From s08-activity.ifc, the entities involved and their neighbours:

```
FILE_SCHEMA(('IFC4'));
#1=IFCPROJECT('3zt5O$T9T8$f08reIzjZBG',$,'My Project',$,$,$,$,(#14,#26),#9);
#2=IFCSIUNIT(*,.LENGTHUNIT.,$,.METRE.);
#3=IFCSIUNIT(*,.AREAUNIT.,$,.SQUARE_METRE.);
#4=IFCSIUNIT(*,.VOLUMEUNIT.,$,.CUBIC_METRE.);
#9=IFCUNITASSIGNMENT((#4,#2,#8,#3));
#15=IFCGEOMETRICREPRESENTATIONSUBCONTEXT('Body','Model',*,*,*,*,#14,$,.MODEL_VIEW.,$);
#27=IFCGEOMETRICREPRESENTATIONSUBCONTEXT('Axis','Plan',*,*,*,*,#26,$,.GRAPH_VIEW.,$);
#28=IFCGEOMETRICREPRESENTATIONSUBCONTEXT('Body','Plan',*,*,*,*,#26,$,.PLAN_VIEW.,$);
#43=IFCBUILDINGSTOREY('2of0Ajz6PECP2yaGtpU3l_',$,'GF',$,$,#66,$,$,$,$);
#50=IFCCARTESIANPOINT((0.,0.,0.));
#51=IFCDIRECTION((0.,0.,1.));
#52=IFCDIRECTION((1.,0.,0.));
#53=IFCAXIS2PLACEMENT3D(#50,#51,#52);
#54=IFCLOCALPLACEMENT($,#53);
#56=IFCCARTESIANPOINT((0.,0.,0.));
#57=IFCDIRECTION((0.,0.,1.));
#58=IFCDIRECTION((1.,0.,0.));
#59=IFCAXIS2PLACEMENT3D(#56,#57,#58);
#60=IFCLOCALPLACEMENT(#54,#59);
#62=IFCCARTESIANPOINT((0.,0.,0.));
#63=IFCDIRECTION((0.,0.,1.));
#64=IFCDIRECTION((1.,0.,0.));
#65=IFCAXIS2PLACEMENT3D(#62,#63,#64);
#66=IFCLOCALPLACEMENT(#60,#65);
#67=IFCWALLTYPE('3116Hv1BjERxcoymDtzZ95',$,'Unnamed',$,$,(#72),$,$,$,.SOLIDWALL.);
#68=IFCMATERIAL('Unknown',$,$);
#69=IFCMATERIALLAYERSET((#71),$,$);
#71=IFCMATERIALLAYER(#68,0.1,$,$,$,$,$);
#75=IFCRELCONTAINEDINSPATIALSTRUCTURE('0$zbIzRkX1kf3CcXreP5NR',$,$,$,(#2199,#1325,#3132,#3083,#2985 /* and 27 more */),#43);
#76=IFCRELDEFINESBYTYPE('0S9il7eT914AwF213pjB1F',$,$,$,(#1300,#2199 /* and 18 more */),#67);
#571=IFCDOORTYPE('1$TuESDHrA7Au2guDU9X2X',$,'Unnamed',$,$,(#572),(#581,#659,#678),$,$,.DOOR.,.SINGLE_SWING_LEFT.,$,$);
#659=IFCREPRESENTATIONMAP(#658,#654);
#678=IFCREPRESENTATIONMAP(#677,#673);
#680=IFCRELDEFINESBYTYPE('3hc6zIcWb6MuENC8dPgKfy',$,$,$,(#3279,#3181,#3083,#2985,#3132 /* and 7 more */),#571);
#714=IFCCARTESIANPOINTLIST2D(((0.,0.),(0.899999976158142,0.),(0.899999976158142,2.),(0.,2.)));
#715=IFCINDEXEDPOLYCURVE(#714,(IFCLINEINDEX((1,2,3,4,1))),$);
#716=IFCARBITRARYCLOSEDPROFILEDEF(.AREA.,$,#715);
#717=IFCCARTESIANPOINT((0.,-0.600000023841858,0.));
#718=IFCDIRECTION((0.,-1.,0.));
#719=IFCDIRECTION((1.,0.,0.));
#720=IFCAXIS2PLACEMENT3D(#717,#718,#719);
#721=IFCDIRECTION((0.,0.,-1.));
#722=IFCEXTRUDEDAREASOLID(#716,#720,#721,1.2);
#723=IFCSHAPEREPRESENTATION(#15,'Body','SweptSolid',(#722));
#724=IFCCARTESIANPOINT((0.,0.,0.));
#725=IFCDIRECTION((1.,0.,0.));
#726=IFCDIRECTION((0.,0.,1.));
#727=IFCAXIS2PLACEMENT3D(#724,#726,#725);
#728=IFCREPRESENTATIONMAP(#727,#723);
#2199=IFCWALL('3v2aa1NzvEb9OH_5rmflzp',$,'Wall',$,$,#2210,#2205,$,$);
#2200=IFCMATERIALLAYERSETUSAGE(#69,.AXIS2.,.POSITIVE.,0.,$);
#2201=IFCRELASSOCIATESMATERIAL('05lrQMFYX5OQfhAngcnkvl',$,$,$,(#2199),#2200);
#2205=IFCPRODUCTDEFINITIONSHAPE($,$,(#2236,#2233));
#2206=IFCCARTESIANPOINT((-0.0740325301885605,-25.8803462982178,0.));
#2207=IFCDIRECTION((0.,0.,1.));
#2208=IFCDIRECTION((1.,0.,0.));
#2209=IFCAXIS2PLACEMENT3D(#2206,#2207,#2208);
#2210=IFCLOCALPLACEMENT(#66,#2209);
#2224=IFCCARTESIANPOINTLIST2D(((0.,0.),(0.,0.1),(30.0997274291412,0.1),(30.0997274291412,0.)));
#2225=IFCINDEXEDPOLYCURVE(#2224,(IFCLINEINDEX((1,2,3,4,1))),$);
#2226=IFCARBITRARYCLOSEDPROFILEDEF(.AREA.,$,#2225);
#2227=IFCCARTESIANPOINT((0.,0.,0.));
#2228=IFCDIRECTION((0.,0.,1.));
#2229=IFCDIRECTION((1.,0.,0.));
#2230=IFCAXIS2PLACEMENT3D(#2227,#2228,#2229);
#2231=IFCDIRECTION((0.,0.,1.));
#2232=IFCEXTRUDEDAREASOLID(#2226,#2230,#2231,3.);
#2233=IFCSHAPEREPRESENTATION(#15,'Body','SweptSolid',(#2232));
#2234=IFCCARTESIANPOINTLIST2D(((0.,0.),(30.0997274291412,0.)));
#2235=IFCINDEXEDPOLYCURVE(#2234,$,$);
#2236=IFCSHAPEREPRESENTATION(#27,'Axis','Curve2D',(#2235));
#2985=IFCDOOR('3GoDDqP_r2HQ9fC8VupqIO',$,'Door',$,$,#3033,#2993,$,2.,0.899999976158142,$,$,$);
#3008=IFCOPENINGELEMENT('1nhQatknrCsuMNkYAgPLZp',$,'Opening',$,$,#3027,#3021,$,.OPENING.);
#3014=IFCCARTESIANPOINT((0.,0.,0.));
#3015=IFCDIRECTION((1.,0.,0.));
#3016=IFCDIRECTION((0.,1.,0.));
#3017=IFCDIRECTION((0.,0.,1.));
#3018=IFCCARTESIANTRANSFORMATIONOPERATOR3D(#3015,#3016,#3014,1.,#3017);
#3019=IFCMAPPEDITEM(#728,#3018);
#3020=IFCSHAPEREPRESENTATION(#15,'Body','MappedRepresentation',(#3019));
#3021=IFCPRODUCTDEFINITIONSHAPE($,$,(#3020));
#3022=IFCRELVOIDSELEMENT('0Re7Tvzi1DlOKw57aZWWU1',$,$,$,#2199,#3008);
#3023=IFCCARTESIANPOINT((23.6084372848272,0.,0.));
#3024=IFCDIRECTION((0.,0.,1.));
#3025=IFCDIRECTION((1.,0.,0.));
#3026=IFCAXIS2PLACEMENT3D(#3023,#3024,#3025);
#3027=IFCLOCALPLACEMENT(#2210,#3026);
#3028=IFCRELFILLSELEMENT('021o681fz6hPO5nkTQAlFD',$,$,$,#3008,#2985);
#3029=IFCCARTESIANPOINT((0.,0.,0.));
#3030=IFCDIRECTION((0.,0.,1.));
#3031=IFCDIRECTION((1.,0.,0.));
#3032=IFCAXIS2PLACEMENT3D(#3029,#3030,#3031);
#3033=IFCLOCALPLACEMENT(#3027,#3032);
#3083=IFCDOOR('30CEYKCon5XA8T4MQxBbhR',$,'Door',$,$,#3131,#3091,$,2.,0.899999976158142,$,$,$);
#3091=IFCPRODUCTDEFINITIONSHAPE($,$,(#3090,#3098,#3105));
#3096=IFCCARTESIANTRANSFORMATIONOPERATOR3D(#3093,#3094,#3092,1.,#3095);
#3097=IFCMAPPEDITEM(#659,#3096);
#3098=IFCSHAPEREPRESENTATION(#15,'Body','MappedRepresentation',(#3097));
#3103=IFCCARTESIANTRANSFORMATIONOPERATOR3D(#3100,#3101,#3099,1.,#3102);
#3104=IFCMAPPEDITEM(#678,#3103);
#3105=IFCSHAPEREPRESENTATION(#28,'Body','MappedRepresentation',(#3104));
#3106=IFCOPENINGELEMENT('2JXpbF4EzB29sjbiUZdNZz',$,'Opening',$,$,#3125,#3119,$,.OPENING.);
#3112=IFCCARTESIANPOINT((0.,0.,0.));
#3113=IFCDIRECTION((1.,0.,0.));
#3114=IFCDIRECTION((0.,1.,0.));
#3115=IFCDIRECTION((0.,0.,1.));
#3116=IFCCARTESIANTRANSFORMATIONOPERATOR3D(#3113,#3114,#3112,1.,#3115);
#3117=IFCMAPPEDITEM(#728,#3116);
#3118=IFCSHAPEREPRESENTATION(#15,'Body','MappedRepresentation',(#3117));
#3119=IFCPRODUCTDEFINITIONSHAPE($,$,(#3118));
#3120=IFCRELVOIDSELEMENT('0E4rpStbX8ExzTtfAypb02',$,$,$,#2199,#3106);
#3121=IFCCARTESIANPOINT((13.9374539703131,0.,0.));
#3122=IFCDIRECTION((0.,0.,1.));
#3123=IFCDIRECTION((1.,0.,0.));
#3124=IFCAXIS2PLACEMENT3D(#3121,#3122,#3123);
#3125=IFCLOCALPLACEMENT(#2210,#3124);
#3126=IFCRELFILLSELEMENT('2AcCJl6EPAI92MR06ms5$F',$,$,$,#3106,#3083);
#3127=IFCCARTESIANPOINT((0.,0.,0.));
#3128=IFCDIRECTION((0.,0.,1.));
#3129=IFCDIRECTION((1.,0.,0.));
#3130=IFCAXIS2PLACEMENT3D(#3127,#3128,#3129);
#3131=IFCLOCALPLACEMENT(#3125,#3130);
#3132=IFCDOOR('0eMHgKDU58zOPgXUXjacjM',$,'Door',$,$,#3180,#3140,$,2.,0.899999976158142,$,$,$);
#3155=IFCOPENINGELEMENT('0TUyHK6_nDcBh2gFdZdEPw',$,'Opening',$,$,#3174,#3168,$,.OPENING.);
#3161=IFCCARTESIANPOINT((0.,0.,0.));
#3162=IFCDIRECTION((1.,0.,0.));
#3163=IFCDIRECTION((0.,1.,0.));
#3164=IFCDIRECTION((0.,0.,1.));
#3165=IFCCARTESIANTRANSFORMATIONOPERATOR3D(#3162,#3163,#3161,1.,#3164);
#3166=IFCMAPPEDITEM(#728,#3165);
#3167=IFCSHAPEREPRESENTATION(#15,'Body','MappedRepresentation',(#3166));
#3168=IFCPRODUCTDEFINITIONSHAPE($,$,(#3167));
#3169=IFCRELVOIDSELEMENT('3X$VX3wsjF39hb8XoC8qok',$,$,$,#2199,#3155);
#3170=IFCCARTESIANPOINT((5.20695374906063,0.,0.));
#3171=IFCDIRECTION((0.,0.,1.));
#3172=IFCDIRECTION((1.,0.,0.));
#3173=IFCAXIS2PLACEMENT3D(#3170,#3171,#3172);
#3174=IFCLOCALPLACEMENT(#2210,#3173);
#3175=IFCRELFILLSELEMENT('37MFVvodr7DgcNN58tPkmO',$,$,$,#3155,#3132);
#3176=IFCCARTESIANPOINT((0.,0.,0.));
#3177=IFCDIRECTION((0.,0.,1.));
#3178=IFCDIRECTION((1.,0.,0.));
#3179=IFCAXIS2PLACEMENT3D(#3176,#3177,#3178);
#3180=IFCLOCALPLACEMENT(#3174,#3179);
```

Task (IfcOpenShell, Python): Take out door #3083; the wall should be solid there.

```python
import ifcopenshell
import ifcopenshell.api.feature
import ifcopenshell.api.root
import ifcopenshell.geom
import ifcopenshell.util.shape

model = ifcopenshell.open("s08-activity.ifc")
settings = ifcopenshell.geom.settings()


def volume(element):
    """Net volume in cubic metres, openings subtracted."""
    shape = ifcopenshell.geom.create_shape(settings, element)
    return ifcopenshell.util.shape.get_volume(shape.geometry)


door = model.by_guid("30CEYKCon5XA8T4MQxBbhR")
opening = door.FillsVoids[0].RelatingOpeningElement
wall = opening.VoidsElements[0].RelatingBuildingElement
before = volume(wall)

ifcopenshell.api.root.remove_product(model, product=door)
ifcopenshell.api.feature.remove_feature(model, feature=opening)

after = volume(wall)

print(f"wall volume {before:.3f} -> {after:.3f} m3")

model.write("s08-activity_edited.ifc")
```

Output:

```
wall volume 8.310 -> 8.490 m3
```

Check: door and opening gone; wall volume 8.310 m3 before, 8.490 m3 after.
